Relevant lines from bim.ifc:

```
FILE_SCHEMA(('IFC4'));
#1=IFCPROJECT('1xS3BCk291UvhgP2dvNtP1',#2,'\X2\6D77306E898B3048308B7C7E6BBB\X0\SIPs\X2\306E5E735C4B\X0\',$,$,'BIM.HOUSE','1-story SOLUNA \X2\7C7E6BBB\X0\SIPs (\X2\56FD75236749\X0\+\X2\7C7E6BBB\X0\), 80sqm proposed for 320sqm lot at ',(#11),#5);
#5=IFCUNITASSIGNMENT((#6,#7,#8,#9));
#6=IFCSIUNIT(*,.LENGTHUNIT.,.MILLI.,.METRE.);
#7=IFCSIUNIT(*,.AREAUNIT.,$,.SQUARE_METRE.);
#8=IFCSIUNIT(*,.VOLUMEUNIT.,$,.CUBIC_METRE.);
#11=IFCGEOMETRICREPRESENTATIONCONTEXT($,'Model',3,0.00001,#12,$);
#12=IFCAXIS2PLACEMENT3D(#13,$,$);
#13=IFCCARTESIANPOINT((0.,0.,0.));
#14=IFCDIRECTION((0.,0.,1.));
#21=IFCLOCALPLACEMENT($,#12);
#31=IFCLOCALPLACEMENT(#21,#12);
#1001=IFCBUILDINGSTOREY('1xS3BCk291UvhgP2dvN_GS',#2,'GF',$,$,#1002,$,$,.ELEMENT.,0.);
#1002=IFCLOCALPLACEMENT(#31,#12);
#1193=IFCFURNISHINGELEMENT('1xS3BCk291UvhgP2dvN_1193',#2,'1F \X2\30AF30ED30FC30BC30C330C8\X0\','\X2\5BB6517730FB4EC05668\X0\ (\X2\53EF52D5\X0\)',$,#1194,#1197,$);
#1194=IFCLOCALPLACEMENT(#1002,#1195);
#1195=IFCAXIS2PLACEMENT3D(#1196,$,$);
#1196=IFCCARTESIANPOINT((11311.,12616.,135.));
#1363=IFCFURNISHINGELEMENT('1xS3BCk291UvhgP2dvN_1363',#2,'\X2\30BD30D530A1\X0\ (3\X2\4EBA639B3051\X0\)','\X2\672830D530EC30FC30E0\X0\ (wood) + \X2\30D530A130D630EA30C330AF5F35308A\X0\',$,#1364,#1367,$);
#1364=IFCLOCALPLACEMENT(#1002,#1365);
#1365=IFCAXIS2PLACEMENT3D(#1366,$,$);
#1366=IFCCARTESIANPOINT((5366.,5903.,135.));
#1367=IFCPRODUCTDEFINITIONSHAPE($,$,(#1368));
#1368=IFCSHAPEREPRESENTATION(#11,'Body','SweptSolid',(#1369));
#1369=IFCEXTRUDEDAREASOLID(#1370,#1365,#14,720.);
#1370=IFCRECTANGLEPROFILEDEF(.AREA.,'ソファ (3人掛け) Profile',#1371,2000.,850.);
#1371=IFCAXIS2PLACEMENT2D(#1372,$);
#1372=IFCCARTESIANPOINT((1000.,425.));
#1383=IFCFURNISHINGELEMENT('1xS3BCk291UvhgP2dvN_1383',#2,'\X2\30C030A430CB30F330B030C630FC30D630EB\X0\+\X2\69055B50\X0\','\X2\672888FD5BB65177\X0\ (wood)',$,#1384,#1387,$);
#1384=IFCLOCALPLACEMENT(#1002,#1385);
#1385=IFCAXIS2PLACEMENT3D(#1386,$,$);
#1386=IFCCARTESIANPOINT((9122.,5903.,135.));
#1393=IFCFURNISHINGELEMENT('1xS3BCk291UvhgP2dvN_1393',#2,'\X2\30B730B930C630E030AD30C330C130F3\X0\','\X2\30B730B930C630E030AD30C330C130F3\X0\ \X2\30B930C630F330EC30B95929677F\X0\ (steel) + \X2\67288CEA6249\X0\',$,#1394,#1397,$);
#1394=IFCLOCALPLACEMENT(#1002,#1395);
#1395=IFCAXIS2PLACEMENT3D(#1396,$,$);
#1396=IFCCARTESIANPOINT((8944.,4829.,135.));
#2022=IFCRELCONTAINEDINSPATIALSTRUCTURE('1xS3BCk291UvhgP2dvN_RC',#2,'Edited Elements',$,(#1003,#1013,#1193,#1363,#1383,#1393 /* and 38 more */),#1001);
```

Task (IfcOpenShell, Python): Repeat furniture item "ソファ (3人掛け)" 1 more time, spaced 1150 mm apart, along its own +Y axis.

```python
import ifcopenshell
import ifcopenshell.api.geometry
import ifcopenshell.api.root
import ifcopenshell.util.element
import ifcopenshell.util.placement

model = ifcopenshell.open("bim.ifc")


def reuse_history(source, copy):
    """copy_class also copies each property set's owner history, people and application; keep the originals."""
    for rel in copy.IsDefinedBy:
        if rel.is_a("IfcRelDefinesByProperties") and (history := rel.RelatingPropertyDefinition.OwnerHistory):
            rel.RelatingPropertyDefinition.OwnerHistory = source.OwnerHistory
            ifcopenshell.util.element.remove_deep2(model, history)


source = model.by_id(1363)
base = ifcopenshell.util.placement.get_local_placement(source.ObjectPlacement)
step = base[:3, 1] * 1150.0

for i in range(1, 2):
    copy = ifcopenshell.api.root.copy_class(model, product=source)
    copy.Representation = ifcopenshell.util.element.copy_deep(
        model, source.Representation, exclude=["IfcGeometricRepresentationContext", "IfcRepresentationMap"]
    )
    reuse_history(source, copy)
    matrix = base.copy()
    matrix[:3, 3] += i * step
    print("added at", matrix[:3, 3].round(3) + 0.0)
    ifcopenshell.api.geometry.edit_object_placement(model, product=copy, matrix=matrix, is_si=False)

model.write("bim_v2.ifc")
```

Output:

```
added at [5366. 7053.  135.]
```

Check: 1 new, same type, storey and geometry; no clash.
